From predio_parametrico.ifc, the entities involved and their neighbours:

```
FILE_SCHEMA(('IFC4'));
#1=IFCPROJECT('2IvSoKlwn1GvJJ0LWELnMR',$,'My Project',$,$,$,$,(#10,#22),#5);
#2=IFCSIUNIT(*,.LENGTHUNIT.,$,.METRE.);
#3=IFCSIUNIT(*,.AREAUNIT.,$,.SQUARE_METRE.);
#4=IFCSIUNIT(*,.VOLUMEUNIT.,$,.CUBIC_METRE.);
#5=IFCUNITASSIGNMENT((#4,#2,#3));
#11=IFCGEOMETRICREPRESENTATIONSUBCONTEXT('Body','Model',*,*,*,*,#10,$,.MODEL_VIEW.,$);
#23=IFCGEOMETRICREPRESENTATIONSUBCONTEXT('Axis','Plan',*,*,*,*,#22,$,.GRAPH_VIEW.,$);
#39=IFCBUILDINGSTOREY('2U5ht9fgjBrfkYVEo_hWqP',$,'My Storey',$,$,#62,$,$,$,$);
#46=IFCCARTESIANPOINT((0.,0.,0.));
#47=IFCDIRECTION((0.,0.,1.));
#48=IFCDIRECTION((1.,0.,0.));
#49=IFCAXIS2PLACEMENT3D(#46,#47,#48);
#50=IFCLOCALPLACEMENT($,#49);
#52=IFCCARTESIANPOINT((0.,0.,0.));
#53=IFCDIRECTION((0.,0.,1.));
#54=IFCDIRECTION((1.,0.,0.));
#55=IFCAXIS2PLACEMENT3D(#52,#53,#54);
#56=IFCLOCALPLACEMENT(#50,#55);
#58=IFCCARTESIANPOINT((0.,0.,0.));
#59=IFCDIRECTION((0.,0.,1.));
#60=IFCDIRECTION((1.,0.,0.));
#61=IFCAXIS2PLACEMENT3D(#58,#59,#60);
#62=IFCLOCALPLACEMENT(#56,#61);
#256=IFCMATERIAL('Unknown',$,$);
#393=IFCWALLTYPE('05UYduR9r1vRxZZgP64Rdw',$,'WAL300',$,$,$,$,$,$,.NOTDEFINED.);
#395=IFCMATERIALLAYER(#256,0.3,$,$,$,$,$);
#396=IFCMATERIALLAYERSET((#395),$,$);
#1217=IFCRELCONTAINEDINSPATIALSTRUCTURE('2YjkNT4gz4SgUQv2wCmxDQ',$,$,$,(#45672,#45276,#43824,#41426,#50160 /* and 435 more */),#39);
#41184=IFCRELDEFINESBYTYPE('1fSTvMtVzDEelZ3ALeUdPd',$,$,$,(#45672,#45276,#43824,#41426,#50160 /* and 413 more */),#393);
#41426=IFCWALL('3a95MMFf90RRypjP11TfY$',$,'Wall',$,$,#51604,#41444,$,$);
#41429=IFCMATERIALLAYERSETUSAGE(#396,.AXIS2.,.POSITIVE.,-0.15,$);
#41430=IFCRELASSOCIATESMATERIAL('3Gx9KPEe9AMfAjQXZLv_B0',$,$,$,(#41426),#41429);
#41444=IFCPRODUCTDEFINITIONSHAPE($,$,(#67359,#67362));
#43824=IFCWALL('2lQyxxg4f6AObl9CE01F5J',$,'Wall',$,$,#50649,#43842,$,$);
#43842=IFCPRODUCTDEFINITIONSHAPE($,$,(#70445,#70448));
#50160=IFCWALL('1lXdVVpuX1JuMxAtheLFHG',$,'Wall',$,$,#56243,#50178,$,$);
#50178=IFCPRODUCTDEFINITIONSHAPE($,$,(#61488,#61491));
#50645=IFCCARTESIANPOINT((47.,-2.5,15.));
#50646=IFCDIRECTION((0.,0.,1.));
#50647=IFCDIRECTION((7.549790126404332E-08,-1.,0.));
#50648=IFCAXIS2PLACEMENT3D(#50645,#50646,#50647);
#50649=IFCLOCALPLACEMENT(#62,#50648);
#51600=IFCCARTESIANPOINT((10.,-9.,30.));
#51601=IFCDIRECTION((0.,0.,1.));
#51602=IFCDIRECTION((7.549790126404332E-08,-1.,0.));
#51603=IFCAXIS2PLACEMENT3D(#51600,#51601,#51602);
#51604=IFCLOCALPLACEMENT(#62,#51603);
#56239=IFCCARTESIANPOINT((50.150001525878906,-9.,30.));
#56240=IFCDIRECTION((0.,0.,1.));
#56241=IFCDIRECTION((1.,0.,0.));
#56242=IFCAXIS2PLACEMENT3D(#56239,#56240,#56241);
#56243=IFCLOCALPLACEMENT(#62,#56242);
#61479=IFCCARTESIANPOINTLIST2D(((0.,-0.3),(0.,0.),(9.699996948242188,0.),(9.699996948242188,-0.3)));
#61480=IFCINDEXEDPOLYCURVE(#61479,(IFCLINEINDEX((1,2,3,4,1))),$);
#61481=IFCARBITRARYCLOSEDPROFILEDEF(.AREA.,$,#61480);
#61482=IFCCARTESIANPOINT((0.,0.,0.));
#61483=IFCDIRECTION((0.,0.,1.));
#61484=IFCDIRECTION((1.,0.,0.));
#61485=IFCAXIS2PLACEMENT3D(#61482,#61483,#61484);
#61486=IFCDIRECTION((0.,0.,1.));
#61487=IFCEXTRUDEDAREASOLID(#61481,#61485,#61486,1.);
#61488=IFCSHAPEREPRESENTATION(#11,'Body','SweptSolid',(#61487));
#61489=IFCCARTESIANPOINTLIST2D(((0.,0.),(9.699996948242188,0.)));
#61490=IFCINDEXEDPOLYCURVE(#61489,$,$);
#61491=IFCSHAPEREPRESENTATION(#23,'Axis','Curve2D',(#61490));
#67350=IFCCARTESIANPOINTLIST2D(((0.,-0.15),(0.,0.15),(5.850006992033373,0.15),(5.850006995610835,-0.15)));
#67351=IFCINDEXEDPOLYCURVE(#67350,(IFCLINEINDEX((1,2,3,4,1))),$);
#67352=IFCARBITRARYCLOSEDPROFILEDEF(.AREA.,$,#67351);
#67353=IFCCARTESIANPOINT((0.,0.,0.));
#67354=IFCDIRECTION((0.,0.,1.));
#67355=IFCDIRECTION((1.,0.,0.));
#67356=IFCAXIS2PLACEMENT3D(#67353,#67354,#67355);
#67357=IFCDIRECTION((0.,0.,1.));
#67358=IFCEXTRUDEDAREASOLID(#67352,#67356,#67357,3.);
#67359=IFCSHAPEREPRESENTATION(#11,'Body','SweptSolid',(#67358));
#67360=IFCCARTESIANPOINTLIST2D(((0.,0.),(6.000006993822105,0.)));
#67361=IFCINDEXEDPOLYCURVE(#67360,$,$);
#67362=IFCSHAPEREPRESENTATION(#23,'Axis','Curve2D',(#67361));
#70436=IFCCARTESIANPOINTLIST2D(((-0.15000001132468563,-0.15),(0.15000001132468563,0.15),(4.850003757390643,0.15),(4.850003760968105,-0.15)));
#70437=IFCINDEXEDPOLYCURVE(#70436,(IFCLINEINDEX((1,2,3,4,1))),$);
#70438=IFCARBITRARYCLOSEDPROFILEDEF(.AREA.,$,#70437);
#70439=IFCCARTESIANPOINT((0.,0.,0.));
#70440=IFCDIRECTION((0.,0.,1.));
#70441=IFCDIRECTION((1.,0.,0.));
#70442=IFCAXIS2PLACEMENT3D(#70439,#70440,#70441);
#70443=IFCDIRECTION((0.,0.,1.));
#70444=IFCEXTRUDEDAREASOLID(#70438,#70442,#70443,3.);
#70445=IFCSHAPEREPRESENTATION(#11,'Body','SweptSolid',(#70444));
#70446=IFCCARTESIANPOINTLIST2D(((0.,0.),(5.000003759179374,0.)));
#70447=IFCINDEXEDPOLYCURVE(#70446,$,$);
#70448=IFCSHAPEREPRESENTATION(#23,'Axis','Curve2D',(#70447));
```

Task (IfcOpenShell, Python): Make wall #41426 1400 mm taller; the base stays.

```python
import ifcopenshell
import ifcopenshell.geom
import ifcopenshell.util.representation
import ifcopenshell.util.shape

model = ifcopenshell.open("predio_parametrico.ifc")
settings = ifcopenshell.geom.settings()


def volume(element):
    """Net volume in cubic metres, openings subtracted."""
    shape = ifcopenshell.geom.create_shape(settings, element)
    return ifcopenshell.util.shape.get_volume(shape.geometry)


wall = model.by_guid("3a95MMFf90RRypjP11TfY$")
before = volume(wall)

body = ifcopenshell.util.representation.get_representation(wall, "Model", "Body")
solid = body.Items[0]
old_height = solid.Depth
solid.Depth += 1.4
after = volume(wall)

print(f"height {old_height:g} -> {solid.Depth:g}, volume {before:.3f} -> {after:.3f} m3")

model.write("predio_parametrico-out.ifc")
```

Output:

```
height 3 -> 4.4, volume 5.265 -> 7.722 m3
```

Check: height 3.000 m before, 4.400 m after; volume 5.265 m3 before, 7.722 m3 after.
